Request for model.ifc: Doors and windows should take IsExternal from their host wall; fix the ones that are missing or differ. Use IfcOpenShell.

First a look at what the model holds.

```python
import ifcopenshell
import ifcopenshell.util.element

model = ifcopenshell.open("model.ifc")
print(model.schema)
seen = {}
for e in model.by_type("IfcDoor") + model.by_type("IfcWindow"):
    if not e.FillsVoids:
        continue
    host = e.FillsVoids[0].RelatingOpeningElement.VoidsElements[0].RelatingBuildingElement
    own = ifcopenshell.util.element.get_pset(e, f"Pset_{e.is_a()[3:].removesuffix('StandardCase')}Common", "IsExternal")
    wall = ifcopenshell.util.element.get_pset(host, "Pset_WallCommon", "IsExternal")
    seen[e.is_a(), own, wall] = seen.get((e.is_a(), own, wall), 0) + 1
for (cls, own, wall), count in sorted(seen.items(), key=str):
    print(count, cls, "IsExternal:", own, "| host wall:", wall)
```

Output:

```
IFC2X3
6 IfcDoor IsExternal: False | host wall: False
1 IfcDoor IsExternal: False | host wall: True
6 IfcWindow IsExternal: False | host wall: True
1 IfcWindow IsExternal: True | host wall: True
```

```python
import ifcopenshell
import ifcopenshell.api.pset
import ifcopenshell.util.element

model = ifcopenshell.open("model.ifc")

count = 0
for ifc_class, pset_name in (("IfcDoor", "Pset_DoorCommon"), ("IfcWindow", "Pset_WindowCommon")):
    for e in model.by_type(ifc_class):
        if not e.FillsVoids:
            continue
        host = e.FillsVoids[0].RelatingOpeningElement.VoidsElements[0].RelatingBuildingElement
        external = ifcopenshell.util.element.get_pset(host, "Pset_WallCommon", "IsExternal")
        if external is None or ifcopenshell.util.element.get_pset(e, pset_name, "IsExternal") == external:
            continue
        pset = ifcopenshell.api.pset.add_pset(model, product=e, name=pset_name)
        ifcopenshell.api.pset.edit_pset(model, pset=pset, properties={"IsExternal": external})
        count += 1

print(count, "updated")

model.write("model_v2.ifc")
```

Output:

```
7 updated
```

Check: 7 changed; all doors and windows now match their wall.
